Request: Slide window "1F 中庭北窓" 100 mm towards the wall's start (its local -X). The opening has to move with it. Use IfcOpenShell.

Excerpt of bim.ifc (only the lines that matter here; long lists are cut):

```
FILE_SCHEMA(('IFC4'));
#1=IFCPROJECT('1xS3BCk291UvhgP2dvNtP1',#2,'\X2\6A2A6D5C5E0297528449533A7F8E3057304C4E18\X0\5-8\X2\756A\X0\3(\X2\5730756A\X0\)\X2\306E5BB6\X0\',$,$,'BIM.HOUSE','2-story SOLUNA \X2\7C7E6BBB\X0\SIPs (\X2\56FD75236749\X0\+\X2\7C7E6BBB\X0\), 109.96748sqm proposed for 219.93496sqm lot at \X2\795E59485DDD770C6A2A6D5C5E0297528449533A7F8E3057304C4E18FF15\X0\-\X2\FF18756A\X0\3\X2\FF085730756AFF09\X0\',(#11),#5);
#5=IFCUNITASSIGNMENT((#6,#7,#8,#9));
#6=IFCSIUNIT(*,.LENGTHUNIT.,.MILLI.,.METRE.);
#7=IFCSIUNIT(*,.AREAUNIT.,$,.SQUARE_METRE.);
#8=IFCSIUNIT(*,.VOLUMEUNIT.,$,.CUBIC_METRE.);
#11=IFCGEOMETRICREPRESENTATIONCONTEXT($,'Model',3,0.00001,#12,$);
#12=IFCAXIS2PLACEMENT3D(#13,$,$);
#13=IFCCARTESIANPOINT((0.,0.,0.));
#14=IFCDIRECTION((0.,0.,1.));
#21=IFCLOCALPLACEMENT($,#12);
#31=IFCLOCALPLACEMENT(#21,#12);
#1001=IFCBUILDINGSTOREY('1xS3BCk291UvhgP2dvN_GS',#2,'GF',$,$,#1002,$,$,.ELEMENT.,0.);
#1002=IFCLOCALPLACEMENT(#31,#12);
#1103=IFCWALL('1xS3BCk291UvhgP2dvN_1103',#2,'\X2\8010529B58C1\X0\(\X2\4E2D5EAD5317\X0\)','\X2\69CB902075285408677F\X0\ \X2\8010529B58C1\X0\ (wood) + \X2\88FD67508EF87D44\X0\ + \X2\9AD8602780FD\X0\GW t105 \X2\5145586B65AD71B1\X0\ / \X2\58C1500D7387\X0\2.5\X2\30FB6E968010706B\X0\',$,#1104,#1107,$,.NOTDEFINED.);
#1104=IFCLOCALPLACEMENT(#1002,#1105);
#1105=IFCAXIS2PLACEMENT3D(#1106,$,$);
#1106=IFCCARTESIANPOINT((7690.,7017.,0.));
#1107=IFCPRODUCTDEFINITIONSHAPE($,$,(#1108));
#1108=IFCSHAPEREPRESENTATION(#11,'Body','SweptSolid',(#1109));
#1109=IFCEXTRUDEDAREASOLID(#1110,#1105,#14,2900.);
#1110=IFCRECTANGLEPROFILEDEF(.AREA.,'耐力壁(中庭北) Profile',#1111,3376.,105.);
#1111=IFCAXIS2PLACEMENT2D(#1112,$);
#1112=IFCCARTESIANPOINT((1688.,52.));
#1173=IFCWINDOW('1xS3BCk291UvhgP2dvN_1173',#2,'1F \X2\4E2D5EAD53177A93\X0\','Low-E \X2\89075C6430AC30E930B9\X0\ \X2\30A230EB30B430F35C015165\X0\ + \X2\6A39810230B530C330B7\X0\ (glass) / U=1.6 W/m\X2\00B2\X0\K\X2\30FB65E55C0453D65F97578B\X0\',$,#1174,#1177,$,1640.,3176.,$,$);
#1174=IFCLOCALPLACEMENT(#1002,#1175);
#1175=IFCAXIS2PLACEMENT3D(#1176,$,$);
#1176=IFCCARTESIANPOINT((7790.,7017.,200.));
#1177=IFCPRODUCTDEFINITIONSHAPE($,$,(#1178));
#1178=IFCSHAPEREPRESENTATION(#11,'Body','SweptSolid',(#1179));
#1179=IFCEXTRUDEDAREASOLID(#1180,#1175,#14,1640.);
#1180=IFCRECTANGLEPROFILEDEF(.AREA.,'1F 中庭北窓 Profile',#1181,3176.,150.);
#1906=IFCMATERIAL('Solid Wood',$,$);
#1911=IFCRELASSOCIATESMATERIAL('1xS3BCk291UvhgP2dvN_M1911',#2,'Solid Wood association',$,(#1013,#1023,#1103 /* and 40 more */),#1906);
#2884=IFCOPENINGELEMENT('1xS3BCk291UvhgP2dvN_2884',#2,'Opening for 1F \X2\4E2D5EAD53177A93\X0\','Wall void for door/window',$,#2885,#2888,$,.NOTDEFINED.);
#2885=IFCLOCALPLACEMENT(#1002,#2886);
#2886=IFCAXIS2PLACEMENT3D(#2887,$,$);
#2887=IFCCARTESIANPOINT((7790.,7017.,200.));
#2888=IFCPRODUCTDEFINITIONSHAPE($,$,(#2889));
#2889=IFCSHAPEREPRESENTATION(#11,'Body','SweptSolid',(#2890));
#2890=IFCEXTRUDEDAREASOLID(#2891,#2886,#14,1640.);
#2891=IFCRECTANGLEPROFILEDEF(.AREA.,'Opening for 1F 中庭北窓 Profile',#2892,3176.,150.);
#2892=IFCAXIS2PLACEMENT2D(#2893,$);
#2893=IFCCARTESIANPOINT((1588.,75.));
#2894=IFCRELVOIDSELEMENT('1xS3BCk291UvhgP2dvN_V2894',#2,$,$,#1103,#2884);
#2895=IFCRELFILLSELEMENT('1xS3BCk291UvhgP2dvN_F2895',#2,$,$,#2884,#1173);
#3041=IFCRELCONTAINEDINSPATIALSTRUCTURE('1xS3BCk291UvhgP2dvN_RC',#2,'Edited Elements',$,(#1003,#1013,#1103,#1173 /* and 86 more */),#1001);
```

```python
import ifcopenshell
import ifcopenshell.api.geometry
import ifcopenshell.util.placement
import ifcopenshell.util.unit

model = ifcopenshell.open("bim.ifc")
unit_scale = ifcopenshell.util.unit.calculate_unit_scale(model)

window = model.by_guid("1xS3BCk291UvhgP2dvN_1173")
opening = window.FillsVoids[0].RelatingOpeningElement
wall = opening.VoidsElements[0].RelatingBuildingElement

wall_matrix = ifcopenshell.util.placement.get_local_placement(wall.ObjectPlacement)
shift = wall_matrix[:3, 0] * -0.1 / unit_scale
before = ifcopenshell.util.placement.get_local_placement(window.ObjectPlacement)[:3, 3].copy()

# The window is not placed relative to its opening, so move both.
for product in (opening, window):
    matrix = ifcopenshell.util.placement.get_local_placement(product.ObjectPlacement)
    matrix[:3, 3] += shift
    ifcopenshell.api.geometry.edit_object_placement(model, product=product, matrix=matrix, is_si=False)

after = ifcopenshell.util.placement.get_local_placement(window.ObjectPlacement)[:3, 3]
print("window moved by", (after - before).round(3) + 0.0)

model.write("bim_v2.ifc")
```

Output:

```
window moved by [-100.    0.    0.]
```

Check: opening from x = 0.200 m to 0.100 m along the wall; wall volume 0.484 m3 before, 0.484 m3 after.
